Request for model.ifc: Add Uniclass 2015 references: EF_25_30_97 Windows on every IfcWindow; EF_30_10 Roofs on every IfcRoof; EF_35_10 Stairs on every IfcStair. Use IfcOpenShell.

First a look at what the model holds.

```python
import ifcopenshell

model = ifcopenshell.open("model.ifc")
print(model.schema)
print("classifications:", [c.Name for c in model.by_type("IfcClassification")])
for ifc_class in ("IfcDoor", "IfcRoof", "IfcStair", "IfcWall", "IfcWindow"):
    print(ifc_class, len(model.by_type(ifc_class)))
```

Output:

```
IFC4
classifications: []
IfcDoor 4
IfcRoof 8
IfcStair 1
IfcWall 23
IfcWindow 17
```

```python
import ifcopenshell
import ifcopenshell.api.classification

model = ifcopenshell.open("model.ifc")

system = ifcopenshell.api.classification.add_classification(model, classification="Uniclass 2015")

codes = {
    "IfcWindow": ("EF_25_30_97", "Windows"),
    "IfcRoof": ("EF_30_10", "Roofs"),
    "IfcStair": ("EF_35_10", "Stairs"),
}
for ifc_class, (code, name) in codes.items():
    products = model.by_type(ifc_class)
    ifcopenshell.api.classification.add_reference(
        model, products=products, classification=system, identification=code, name=name
    )
    print(code, len(products))

model.write("model-out.ifc")
```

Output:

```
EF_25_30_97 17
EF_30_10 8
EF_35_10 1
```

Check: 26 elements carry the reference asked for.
